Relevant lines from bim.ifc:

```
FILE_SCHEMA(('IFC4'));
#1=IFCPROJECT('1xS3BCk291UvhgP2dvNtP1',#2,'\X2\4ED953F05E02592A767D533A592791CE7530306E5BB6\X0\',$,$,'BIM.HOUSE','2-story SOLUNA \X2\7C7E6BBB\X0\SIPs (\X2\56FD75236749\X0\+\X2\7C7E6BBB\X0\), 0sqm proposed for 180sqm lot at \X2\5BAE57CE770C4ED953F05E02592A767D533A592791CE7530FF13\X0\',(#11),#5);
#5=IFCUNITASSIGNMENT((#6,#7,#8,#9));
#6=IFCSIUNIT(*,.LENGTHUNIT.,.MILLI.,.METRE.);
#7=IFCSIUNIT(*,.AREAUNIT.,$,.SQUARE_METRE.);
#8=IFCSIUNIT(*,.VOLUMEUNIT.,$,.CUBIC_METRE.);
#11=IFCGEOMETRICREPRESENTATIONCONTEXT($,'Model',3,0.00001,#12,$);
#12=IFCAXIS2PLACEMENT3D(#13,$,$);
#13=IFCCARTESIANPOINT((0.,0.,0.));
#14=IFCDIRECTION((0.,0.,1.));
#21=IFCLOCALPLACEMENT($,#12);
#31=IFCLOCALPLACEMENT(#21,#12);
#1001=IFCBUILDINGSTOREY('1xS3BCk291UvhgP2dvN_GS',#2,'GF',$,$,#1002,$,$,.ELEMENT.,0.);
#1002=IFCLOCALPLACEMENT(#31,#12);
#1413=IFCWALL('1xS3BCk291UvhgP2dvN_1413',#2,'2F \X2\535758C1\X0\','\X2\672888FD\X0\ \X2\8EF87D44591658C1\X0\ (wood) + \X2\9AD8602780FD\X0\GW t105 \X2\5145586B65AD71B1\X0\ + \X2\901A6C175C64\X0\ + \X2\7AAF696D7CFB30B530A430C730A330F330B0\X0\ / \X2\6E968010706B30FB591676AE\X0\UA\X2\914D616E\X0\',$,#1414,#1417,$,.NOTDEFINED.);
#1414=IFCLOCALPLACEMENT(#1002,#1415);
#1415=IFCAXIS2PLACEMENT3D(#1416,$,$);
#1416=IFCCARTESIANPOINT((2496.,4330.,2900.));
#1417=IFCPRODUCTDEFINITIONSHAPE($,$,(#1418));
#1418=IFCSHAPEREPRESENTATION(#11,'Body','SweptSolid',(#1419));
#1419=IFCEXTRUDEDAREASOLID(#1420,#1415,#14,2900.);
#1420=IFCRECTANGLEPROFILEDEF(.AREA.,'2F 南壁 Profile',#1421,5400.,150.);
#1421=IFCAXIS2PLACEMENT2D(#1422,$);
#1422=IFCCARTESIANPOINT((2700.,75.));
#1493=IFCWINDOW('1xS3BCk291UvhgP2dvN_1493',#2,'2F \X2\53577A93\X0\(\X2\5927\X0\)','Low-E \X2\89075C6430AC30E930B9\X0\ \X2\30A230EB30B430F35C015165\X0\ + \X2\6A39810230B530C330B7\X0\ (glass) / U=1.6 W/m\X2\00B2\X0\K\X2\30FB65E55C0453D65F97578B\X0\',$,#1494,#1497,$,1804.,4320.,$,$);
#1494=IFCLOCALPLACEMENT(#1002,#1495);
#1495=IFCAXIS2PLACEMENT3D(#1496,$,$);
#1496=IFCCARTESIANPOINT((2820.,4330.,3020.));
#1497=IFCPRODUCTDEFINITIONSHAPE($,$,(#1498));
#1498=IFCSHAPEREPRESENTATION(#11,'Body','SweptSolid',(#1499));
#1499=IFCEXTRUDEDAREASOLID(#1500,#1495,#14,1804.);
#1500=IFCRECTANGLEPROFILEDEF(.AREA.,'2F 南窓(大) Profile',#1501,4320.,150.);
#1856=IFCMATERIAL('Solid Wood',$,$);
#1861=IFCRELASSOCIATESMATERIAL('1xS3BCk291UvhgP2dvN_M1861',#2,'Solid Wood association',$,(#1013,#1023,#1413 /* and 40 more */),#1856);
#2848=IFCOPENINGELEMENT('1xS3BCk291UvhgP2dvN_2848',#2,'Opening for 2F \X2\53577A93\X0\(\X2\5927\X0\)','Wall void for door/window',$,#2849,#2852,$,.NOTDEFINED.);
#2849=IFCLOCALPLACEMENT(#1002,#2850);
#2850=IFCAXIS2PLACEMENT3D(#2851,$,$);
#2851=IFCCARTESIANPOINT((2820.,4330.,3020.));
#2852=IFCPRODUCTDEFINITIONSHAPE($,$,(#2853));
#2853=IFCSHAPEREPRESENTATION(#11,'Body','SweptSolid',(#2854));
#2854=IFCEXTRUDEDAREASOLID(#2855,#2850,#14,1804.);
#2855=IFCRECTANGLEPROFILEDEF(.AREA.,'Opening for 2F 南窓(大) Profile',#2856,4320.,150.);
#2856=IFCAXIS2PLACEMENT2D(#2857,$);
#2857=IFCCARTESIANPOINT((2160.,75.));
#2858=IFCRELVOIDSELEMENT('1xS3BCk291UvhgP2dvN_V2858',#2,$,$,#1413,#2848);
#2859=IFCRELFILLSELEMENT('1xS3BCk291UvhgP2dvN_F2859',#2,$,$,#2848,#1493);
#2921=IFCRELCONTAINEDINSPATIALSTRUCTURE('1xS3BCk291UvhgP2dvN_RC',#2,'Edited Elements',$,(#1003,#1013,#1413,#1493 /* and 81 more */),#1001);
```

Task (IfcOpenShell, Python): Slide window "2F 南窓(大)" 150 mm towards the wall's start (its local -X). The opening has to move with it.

```python
import ifcopenshell
import ifcopenshell.api.geometry
import ifcopenshell.util.placement

model = ifcopenshell.open("bim.ifc")

window = model.by_guid("1xS3BCk291UvhgP2dvN_1493")
opening = window.FillsVoids[0].RelatingOpeningElement
wall = opening.VoidsElements[0].RelatingBuildingElement

wall_matrix = ifcopenshell.util.placement.get_local_placement(wall.ObjectPlacement)
shift = wall_matrix[:3, 0] * -150.0
before = ifcopenshell.util.placement.get_local_placement(window.ObjectPlacement)[:3, 3].copy()

# The window is not placed relative to its opening, so move both.
for product in (opening, window):
    matrix = ifcopenshell.util.placement.get_local_placement(product.ObjectPlacement)
    matrix[:3, 3] += shift
    ifcopenshell.api.geometry.edit_object_placement(model, product=product, matrix=matrix, is_si=False)

after = ifcopenshell.util.placement.get_local_placement(window.ObjectPlacement)[:3, 3]
print("window moved by", (after - before).round(3) + 0.0)

model.write("bim-out.ifc")
```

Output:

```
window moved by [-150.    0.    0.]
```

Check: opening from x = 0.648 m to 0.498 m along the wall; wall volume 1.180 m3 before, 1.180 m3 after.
